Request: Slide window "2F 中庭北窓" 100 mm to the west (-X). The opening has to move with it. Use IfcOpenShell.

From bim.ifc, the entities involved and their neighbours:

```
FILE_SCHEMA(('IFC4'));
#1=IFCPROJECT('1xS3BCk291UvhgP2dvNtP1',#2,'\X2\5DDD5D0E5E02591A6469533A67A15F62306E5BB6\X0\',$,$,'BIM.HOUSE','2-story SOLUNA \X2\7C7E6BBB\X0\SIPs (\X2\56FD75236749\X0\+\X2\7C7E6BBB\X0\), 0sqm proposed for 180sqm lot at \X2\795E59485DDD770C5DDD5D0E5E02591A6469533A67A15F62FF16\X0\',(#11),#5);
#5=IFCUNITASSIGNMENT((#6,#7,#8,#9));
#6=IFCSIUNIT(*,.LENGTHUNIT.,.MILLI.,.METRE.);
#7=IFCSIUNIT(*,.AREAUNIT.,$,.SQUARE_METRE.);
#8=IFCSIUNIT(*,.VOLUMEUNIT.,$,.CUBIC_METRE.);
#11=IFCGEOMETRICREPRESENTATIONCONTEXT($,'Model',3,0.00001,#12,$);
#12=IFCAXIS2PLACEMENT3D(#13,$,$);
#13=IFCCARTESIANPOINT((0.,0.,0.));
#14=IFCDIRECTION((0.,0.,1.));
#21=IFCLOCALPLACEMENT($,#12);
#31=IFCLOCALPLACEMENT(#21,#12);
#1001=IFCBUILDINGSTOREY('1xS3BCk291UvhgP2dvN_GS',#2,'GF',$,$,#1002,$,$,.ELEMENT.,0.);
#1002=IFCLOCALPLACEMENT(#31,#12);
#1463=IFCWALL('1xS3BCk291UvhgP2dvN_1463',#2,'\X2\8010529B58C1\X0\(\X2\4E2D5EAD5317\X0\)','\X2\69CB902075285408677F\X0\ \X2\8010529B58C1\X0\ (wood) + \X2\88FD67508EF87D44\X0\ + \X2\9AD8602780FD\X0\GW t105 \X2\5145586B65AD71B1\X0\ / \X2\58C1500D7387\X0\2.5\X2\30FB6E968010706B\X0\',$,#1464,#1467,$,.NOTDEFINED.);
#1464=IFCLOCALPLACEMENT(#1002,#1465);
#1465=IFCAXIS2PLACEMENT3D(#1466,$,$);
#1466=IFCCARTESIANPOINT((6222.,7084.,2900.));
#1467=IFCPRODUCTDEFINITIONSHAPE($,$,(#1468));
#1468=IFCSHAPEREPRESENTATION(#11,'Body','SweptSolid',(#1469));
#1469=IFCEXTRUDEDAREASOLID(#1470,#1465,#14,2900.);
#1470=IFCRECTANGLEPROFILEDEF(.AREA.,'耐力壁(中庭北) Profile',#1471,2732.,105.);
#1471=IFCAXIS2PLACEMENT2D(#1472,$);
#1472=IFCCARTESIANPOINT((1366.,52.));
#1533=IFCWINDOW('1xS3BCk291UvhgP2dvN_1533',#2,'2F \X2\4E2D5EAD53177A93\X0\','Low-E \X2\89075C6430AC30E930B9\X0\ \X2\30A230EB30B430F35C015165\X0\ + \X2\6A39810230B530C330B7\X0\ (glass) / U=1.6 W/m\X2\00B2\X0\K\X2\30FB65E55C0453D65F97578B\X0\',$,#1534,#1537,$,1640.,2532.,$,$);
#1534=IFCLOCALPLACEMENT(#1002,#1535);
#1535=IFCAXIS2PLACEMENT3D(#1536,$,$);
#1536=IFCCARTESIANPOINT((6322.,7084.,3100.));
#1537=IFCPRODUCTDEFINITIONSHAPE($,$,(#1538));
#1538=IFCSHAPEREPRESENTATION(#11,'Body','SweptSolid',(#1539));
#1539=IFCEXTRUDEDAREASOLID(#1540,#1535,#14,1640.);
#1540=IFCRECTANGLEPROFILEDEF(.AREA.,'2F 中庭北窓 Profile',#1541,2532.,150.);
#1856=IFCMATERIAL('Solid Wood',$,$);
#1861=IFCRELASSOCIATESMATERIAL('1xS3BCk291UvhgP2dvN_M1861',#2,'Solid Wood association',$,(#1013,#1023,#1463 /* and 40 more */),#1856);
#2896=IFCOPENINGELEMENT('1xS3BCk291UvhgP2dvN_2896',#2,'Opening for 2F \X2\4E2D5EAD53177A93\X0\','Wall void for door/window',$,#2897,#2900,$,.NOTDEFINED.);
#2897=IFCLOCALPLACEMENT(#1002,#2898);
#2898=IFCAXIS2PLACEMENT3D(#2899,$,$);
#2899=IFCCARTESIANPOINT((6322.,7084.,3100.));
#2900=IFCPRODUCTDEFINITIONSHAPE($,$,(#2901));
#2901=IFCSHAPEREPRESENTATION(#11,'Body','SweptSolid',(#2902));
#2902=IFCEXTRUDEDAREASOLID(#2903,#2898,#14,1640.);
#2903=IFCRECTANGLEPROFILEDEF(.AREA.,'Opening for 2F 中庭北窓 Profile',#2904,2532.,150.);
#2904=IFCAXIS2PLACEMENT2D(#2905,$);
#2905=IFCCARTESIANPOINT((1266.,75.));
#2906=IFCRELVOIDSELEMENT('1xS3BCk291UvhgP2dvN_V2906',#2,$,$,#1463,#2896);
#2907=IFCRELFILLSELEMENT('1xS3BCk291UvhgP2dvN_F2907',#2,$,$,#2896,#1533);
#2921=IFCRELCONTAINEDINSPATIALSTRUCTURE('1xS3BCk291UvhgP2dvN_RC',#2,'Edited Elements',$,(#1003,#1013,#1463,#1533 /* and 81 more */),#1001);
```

```python
import ifcopenshell
import ifcopenshell.api.geometry
import ifcopenshell.util.placement
import ifcopenshell.util.unit

model = ifcopenshell.open("bim.ifc")
unit_scale = ifcopenshell.util.unit.calculate_unit_scale(model)

window = model.by_id(1533)
opening = window.FillsVoids[0].RelatingOpeningElement
wall = opening.VoidsElements[0].RelatingBuildingElement

wall_matrix = ifcopenshell.util.placement.get_local_placement(wall.ObjectPlacement)
shift = wall_matrix[:3, 0] * -0.1 / unit_scale
before = ifcopenshell.util.placement.get_local_placement(window.ObjectPlacement)[:3, 3].copy()

# The window is not placed relative to its opening, so move both.
for product in (opening, window):
    matrix = ifcopenshell.util.placement.get_local_placement(product.ObjectPlacement)
    matrix[:3, 3] += shift
    ifcopenshell.api.geometry.edit_object_placement(model, product=product, matrix=matrix, is_si=False)

after = ifcopenshell.util.placement.get_local_placement(window.ObjectPlacement)[:3, 3]
print("window moved by", (after - before).round(3) + 0.0)

model.write("bim_rev.ifc")
```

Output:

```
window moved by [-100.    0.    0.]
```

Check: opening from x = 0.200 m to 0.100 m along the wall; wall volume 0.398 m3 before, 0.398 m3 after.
